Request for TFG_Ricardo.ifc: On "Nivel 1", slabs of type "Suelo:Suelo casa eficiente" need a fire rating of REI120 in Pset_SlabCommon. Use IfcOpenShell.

First a look at what the model holds.

```python
import ifcopenshell
import ifcopenshell.util.element

model = ifcopenshell.open("TFG_Ricardo.ifc")
print(model.schema)
storey = next(s for s in model.by_type("IfcBuildingStorey") if s.Name == "Nivel 1")
slabs = [e for e in ifcopenshell.util.element.get_decomposition(storey) if e.is_a("IfcSlab")]
seen = {}
for e in slabs:
    element_type = ifcopenshell.util.element.get_type(e)
    key = (element_type.Name if element_type != e and element_type else None, ifcopenshell.util.element.get_pset(e, "Pset_SlabCommon", "FireRating"))
    seen[key] = seen.get(key, 0) + 1
for (name, value), count in sorted(seen.items(), key=str):
    print(count, "x", name, "|", value)
```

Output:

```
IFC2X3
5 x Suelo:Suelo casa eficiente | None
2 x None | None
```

```python
import ifcopenshell
import ifcopenshell.api.pset
import ifcopenshell.util.element

model = ifcopenshell.open("TFG_Ricardo.ifc")

storey = next(s for s in model.by_type("IfcBuildingStorey") if s.Name == "Nivel 1")
slabs = [e for e in ifcopenshell.util.element.get_decomposition(storey) if e.is_a("IfcSlab")]

count = 0
for e in slabs:
    element_type = ifcopenshell.util.element.get_type(e)
    if element_type in (None, e) or element_type.Name != "Suelo:Suelo casa eficiente":
        continue
    # add_pset returns the element's existing set when there is one.
    pset = ifcopenshell.api.pset.add_pset(model, product=e, name="Pset_SlabCommon")
    ifcopenshell.api.pset.edit_pset(model, pset=pset, properties={"FireRating": "REI120"})
    count += 1

print(count, "slabs updated")

model.write("TFG_Ricardo_v2.ifc")
```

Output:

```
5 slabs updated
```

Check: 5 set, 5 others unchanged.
